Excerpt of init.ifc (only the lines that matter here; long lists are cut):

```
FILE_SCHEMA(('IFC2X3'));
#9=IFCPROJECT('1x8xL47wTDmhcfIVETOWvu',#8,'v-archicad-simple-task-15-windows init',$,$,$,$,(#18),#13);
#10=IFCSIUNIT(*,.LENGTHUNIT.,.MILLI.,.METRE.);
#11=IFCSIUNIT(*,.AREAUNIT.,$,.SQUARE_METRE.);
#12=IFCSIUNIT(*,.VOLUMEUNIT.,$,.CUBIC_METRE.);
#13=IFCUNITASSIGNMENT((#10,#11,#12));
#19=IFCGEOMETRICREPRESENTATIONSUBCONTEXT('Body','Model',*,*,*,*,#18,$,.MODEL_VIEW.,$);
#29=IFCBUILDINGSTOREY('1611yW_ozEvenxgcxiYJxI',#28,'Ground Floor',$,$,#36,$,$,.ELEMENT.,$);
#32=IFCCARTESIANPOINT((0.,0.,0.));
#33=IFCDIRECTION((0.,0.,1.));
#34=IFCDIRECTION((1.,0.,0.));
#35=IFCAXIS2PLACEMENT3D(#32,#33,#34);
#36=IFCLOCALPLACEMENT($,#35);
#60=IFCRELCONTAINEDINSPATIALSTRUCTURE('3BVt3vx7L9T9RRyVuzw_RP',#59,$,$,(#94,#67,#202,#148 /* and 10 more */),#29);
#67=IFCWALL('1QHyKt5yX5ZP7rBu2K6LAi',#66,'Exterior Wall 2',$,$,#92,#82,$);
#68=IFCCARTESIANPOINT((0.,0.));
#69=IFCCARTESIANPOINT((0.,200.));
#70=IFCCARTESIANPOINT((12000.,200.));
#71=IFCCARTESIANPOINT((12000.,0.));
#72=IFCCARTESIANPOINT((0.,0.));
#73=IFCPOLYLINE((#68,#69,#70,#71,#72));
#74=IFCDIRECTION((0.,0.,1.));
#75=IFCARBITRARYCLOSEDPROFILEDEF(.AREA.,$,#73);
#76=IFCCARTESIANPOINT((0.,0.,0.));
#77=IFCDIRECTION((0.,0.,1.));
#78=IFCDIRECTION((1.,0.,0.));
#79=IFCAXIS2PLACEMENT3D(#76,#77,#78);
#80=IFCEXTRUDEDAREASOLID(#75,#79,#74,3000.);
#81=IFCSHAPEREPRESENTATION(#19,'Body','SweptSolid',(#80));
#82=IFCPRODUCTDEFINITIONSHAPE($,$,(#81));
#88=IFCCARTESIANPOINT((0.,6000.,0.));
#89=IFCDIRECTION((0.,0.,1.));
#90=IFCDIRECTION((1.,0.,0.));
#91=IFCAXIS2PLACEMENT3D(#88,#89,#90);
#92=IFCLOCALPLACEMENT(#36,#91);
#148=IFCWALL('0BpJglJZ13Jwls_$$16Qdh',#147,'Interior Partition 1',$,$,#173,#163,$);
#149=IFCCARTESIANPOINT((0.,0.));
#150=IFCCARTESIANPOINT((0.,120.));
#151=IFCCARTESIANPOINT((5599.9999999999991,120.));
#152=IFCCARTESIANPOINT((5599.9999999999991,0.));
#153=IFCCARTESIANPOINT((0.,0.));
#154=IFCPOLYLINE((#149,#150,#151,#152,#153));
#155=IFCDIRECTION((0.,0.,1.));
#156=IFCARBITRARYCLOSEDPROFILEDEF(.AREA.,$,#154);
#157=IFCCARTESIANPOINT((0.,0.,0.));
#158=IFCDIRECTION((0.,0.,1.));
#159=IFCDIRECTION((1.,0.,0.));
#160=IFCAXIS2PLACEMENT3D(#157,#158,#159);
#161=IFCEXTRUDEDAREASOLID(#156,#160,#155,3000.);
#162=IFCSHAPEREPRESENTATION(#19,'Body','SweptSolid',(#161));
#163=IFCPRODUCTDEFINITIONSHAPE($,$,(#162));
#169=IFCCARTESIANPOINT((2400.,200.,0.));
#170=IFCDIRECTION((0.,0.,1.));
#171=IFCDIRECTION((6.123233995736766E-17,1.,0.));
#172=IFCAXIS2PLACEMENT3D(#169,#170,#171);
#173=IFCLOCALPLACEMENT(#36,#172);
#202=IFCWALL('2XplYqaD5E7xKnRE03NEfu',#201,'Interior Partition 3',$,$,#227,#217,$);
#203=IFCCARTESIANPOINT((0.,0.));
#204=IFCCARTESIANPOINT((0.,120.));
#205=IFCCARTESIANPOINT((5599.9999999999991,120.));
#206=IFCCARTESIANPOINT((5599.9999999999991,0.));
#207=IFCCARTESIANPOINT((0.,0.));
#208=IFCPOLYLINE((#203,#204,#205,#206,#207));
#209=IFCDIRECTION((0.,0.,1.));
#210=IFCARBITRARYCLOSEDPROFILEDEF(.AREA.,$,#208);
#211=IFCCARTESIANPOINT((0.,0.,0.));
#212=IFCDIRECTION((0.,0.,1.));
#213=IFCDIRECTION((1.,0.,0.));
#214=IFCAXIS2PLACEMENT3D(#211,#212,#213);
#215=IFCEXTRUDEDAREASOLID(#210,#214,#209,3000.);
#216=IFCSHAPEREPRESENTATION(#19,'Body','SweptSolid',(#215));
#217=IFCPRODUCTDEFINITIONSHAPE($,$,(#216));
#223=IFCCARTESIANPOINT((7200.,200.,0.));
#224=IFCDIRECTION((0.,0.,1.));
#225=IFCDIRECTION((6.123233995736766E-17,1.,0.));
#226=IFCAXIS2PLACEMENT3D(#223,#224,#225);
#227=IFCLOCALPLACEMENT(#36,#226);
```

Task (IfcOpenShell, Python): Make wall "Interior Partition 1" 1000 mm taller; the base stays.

```python
import ifcopenshell
import ifcopenshell.geom
import ifcopenshell.util.representation
import ifcopenshell.util.shape
import ifcopenshell.util.unit

model = ifcopenshell.open("init.ifc")
unit_scale = ifcopenshell.util.unit.calculate_unit_scale(model)
settings = ifcopenshell.geom.settings()


def volume(element):
    """Net volume in cubic metres, openings subtracted."""
    shape = ifcopenshell.geom.create_shape(settings, element)
    return ifcopenshell.util.shape.get_volume(shape.geometry)


wall = model.by_guid("0BpJglJZ13Jwls_$$16Qdh")
before = volume(wall)

body = ifcopenshell.util.representation.get_representation(wall, "Model", "Body")
solid = body.Items[0]
old_height = solid.Depth
solid.Depth += 1 / unit_scale
after = volume(wall)

print(f"height {old_height:g} -> {solid.Depth:g}, volume {before:.3f} -> {after:.3f} m3")

model.write("init_updated.ifc")
```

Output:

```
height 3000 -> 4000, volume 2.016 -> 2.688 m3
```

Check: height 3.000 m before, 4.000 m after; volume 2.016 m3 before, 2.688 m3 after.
